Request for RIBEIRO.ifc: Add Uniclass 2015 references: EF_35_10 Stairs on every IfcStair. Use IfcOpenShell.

First a look at what the model holds.

```python
import ifcopenshell

model = ifcopenshell.open("RIBEIRO.ifc")
print(model.schema)
print("classifications:", [c.Name for c in model.by_type("IfcClassification")])
for ifc_class in ("IfcDoor", "IfcRoof", "IfcStair", "IfcWall", "IfcWindow"):
    print(ifc_class, len(model.by_type(ifc_class)))
```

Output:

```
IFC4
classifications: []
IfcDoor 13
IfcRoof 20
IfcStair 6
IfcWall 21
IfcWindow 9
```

```python
import ifcopenshell
import ifcopenshell.api.classification

model = ifcopenshell.open("RIBEIRO.ifc")

system = ifcopenshell.api.classification.add_classification(model, classification="Uniclass 2015")

codes = {
    "IfcStair": ("EF_35_10", "Stairs"),
}
for ifc_class, (code, name) in codes.items():
    products = model.by_type(ifc_class)
    ifcopenshell.api.classification.add_reference(
        model, products=products, classification=system, identification=code, name=name
    )
    print(code, len(products))

model.write("RIBEIRO_updated.ifc")
```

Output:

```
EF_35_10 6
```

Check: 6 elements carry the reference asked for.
